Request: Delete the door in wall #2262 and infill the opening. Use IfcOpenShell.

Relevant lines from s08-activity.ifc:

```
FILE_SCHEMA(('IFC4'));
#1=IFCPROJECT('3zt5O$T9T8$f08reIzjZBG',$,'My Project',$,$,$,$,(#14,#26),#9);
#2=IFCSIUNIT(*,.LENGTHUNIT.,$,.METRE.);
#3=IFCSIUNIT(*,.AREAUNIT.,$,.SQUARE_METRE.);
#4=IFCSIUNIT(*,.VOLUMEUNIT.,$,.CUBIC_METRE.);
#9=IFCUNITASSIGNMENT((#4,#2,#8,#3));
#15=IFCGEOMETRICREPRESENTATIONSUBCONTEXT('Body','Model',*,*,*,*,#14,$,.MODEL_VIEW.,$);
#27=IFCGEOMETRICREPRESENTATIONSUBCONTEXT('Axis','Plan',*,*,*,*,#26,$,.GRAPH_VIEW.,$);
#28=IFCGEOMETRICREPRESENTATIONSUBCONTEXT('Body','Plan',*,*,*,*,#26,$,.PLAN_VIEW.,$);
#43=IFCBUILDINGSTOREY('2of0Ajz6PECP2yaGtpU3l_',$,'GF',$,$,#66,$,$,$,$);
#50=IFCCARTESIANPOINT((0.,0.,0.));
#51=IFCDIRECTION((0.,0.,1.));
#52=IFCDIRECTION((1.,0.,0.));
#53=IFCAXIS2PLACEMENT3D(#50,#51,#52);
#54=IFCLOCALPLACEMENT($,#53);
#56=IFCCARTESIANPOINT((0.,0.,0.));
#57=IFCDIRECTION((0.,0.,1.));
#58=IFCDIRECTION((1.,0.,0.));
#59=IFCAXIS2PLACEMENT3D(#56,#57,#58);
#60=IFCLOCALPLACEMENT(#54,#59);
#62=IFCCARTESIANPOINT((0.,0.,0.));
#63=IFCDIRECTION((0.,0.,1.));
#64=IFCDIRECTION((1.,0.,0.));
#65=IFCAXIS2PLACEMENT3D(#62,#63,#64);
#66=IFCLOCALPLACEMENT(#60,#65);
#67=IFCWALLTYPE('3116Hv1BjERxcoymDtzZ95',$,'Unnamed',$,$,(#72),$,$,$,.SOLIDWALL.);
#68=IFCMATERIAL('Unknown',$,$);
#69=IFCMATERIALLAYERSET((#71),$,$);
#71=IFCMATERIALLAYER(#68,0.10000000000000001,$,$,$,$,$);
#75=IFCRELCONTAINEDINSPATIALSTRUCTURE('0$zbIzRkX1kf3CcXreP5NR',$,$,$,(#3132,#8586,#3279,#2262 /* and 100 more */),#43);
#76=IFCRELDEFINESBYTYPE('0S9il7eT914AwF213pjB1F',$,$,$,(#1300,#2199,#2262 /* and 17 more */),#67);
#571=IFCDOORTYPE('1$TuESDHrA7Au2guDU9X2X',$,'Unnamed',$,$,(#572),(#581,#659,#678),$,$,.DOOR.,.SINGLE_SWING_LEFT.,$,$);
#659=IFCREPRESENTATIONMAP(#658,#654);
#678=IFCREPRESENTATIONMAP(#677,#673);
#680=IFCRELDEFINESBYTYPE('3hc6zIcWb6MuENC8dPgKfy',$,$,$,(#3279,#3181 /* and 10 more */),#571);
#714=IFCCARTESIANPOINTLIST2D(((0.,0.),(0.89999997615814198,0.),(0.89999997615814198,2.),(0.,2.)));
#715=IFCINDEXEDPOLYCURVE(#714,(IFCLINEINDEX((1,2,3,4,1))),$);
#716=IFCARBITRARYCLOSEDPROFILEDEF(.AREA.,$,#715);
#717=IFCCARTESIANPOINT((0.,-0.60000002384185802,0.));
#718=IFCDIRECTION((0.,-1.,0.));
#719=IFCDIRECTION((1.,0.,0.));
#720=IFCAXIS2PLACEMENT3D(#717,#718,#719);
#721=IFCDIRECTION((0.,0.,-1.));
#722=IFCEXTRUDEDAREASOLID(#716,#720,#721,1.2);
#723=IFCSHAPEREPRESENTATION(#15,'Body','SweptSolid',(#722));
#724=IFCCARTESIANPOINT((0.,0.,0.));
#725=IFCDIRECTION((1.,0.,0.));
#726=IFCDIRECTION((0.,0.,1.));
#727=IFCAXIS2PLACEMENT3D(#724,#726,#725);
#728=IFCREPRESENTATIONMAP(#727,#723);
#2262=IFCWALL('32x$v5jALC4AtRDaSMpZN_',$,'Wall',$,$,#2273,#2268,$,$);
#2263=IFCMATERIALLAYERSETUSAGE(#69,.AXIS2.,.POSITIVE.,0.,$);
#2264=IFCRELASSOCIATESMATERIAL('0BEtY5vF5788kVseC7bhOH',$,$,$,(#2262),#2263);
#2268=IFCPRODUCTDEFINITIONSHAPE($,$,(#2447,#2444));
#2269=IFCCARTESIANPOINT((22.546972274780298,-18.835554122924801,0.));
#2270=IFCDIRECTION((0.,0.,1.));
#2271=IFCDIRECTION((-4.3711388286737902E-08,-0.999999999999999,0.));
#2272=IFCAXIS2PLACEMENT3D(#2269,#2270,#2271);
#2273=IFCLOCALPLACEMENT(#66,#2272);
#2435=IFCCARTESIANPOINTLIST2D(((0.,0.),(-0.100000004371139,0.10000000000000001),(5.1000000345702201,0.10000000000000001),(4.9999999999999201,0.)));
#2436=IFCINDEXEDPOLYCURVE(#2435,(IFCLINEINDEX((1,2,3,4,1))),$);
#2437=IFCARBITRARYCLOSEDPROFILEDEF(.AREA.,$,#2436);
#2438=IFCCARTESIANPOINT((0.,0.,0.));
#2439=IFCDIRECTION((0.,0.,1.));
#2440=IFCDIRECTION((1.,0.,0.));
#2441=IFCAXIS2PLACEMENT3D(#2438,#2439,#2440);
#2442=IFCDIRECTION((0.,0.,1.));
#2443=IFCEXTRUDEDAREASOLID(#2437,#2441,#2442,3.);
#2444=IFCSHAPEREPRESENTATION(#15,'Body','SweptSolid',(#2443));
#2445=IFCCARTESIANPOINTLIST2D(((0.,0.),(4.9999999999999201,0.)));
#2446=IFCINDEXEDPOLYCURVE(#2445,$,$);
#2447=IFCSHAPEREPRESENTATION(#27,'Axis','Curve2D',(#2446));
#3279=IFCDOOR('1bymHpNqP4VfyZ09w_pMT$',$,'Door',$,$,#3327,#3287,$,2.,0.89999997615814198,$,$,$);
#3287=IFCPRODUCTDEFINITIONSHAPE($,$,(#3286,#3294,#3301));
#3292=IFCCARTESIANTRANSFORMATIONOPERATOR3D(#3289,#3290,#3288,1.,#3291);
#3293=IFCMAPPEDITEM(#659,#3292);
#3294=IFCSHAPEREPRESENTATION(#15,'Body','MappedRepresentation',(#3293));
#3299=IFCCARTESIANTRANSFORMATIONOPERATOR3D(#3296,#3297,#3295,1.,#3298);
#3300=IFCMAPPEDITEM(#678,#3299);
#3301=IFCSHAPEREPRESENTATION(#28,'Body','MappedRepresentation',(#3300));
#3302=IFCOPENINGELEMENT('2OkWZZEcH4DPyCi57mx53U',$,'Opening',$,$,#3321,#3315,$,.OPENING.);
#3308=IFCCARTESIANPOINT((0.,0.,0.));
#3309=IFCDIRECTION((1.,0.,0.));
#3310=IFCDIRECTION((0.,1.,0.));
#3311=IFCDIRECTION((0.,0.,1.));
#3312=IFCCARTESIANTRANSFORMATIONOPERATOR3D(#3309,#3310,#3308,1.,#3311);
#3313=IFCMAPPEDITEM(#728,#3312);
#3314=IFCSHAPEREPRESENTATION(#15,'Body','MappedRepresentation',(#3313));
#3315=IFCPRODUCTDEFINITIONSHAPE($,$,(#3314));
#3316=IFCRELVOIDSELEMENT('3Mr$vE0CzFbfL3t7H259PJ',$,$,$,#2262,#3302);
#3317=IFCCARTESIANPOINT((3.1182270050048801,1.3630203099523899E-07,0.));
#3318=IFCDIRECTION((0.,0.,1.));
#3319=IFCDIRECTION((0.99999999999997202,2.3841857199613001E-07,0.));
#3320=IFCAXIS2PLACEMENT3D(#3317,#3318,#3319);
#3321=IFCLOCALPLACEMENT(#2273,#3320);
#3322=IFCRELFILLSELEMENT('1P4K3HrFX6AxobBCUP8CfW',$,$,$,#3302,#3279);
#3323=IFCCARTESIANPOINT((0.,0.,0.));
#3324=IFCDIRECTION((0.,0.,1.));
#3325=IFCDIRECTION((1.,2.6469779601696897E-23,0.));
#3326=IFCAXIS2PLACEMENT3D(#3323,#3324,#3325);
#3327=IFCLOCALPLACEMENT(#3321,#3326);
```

```python
import ifcopenshell
import ifcopenshell.api.feature
import ifcopenshell.api.root
import ifcopenshell.geom
import ifcopenshell.util.shape

model = ifcopenshell.open("s08-activity.ifc")
settings = ifcopenshell.geom.settings()


def volume(element):
    """Net volume in cubic metres, openings subtracted."""
    shape = ifcopenshell.geom.create_shape(settings, element)
    return ifcopenshell.util.shape.get_volume(shape.geometry)


door = model.by_id(3279)
opening = door.FillsVoids[0].RelatingOpeningElement
wall = opening.VoidsElements[0].RelatingBuildingElement
before = volume(wall)

ifcopenshell.api.root.remove_product(model, product=door)
ifcopenshell.api.feature.remove_feature(model, feature=opening)

after = volume(wall)

print(f"wall volume {before:.3f} -> {after:.3f} m3")

model.write("s08-activity_edited.ifc")
```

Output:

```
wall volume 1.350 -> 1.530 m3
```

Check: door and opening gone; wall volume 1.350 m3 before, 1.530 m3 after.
